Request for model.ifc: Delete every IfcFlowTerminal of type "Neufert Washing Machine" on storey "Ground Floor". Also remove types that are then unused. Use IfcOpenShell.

First a look at what the model holds.

```python
import ifcopenshell
import ifcopenshell.util.element

model = ifcopenshell.open("model.ifc")
print(model.schema)
storey = next(s for s in model.by_type("IfcBuildingStorey") if s.Name == "Ground Floor")
terminals = [e for e in ifcopenshell.util.element.get_decomposition(storey) if e.is_a("IfcFlowTerminal")]
seen = {}
for e in terminals:
    element_type = ifcopenshell.util.element.get_type(e)
    name = element_type.Name if element_type not in (None, e) else None
    seen[name] = seen.get(name, 0) + 1
for name, count in sorted(seen.items(), key=str):
    print(count, "x", name)
```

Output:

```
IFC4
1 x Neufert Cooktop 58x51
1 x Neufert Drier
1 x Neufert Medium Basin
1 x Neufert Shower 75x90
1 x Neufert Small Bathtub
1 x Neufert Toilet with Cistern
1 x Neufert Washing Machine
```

```python
import ifcopenshell
import ifcopenshell.api.root
import ifcopenshell.util.element

model = ifcopenshell.open("model.ifc")

storey = next(s for s in model.by_type("IfcBuildingStorey") if s.Name == "Ground Floor")
terminals = [e for e in ifcopenshell.util.element.get_decomposition(storey) if e.is_a("IfcFlowTerminal")]
targets = [e for e in terminals if (t := ifcopenshell.util.element.get_type(e)) not in (None, e) and t.Name == "Neufert Washing Machine"]
types = {ifcopenshell.util.element.get_type(e) for e in targets} - {None, *targets}

for e in targets:
    ifcopenshell.api.root.remove_product(model, product=e)
print(len(targets), "removed")

unused = [t for t in types if not ifcopenshell.util.element.get_types(t)]
for t in unused:
    ifcopenshell.api.root.remove_product(model, product=t)
print(len(unused), "unused types removed")

model.write("model_v2.ifc")
```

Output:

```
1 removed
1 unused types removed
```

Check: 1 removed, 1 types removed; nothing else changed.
